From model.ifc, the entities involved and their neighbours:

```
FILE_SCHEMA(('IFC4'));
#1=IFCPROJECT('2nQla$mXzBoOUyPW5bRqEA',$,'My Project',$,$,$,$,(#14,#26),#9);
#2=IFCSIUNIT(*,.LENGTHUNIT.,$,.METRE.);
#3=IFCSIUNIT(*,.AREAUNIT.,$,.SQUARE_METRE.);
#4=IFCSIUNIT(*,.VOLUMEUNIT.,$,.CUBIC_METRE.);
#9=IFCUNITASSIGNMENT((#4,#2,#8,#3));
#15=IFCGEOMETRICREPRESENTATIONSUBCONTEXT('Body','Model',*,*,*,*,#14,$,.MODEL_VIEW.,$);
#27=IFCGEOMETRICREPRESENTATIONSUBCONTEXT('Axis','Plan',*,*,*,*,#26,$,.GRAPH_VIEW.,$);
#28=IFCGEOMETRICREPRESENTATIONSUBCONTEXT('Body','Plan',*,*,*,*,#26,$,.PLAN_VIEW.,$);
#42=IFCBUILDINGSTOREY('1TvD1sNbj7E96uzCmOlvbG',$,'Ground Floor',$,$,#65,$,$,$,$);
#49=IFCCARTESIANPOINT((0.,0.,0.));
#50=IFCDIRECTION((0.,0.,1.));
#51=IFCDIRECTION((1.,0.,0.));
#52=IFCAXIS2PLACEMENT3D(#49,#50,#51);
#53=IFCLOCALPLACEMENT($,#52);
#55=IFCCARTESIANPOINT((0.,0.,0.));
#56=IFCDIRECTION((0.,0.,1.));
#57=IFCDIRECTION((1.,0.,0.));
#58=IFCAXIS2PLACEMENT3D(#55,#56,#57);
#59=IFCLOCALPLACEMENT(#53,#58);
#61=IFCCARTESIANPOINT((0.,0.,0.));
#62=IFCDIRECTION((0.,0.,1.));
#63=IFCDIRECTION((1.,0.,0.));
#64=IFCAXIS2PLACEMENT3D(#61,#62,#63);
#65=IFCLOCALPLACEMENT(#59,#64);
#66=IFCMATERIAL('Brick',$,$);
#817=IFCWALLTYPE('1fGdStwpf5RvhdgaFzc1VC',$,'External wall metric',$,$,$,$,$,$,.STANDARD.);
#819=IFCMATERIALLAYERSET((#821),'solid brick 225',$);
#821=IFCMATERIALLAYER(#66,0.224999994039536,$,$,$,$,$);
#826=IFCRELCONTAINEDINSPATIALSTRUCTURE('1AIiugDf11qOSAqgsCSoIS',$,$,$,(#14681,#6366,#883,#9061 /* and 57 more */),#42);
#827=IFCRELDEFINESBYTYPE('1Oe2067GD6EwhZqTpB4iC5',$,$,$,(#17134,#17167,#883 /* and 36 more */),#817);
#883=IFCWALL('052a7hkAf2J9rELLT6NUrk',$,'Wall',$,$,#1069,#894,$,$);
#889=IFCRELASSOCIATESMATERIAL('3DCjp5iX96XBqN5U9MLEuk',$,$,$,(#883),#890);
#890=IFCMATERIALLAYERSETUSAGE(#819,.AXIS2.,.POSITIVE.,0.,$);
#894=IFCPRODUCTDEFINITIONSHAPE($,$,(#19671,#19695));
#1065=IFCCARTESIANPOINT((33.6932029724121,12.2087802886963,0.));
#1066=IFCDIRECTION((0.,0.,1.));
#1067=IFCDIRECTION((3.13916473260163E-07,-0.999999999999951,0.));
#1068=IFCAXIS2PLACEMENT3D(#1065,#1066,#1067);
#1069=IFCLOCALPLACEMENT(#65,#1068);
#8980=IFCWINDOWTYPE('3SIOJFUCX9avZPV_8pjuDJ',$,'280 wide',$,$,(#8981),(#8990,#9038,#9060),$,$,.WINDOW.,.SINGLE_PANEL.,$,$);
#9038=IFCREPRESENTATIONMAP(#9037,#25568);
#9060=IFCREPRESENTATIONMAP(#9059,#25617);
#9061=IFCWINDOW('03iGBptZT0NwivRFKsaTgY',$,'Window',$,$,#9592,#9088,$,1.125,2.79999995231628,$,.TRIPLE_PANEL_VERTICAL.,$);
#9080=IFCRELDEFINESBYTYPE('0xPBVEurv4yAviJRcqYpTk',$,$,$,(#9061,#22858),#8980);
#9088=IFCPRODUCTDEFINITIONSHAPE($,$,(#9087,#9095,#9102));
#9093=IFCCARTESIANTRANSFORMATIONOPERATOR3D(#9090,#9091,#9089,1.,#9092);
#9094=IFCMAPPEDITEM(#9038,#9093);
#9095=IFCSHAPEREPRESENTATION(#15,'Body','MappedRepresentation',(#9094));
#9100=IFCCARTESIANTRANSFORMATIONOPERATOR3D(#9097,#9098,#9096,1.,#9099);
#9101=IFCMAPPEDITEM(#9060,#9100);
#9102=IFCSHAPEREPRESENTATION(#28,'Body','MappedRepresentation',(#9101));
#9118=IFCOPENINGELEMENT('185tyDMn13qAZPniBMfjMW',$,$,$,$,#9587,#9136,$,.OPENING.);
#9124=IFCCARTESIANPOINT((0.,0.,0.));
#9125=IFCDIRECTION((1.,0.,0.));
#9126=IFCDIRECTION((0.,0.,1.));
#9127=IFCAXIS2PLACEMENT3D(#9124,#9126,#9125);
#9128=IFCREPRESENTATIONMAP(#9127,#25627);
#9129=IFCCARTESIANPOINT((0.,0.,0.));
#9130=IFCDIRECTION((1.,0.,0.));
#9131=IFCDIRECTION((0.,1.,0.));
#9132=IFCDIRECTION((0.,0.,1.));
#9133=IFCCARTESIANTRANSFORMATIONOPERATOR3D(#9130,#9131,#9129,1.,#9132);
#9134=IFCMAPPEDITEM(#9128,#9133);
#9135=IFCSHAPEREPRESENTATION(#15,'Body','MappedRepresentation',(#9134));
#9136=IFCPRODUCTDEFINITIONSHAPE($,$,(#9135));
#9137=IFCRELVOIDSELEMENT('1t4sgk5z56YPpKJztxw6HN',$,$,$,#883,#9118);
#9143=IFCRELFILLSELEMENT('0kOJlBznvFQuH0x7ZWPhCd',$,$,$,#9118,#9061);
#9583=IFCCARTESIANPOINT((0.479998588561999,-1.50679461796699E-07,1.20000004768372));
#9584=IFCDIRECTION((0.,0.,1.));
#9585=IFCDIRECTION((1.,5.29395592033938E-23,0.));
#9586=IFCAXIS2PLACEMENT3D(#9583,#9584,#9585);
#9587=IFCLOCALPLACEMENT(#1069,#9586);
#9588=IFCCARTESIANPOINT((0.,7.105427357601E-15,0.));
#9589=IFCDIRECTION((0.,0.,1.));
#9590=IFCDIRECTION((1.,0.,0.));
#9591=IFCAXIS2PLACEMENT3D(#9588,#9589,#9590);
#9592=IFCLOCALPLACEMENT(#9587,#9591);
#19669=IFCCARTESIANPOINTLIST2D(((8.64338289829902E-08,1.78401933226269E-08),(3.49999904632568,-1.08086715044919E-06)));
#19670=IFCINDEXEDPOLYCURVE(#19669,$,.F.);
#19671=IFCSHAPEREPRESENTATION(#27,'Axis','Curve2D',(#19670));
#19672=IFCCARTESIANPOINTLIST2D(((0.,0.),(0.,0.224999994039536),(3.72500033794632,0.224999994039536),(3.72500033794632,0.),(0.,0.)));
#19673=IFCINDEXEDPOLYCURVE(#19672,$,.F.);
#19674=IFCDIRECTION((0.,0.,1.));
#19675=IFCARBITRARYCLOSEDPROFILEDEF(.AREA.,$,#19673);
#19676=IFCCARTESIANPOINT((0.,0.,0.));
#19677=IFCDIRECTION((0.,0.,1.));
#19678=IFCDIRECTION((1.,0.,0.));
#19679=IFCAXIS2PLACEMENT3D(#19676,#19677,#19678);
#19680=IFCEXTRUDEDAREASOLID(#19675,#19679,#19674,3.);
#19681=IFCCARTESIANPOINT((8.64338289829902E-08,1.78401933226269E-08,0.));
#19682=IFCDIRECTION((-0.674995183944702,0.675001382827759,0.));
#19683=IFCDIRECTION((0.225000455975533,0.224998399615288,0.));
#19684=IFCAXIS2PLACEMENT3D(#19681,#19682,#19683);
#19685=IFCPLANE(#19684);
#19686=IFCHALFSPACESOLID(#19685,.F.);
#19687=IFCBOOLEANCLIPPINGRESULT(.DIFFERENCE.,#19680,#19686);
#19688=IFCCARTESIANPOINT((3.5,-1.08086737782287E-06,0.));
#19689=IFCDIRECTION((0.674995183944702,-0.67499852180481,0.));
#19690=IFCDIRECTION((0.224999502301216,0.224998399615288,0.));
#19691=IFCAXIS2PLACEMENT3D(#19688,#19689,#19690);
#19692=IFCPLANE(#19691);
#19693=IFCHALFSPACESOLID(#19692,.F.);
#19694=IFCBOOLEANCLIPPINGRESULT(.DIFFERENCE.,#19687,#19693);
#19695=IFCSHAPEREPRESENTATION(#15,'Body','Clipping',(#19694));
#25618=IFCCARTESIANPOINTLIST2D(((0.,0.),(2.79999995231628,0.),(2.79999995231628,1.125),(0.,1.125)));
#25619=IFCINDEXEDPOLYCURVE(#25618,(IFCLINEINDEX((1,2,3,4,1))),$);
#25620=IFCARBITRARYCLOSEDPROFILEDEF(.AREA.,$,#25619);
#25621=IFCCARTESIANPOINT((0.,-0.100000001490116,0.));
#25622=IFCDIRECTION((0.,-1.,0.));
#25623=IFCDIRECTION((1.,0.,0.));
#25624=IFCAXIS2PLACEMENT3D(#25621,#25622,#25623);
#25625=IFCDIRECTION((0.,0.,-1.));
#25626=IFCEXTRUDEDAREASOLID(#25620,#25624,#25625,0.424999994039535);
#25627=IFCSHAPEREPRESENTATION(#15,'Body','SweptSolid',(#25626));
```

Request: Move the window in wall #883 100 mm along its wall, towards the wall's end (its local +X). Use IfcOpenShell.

```python
import ifcopenshell
import ifcopenshell.api.geometry
import ifcopenshell.util.placement
import ifcopenshell.util.unit

model = ifcopenshell.open("model.ifc")
unit_scale = ifcopenshell.util.unit.calculate_unit_scale(model)

window = model.by_guid("03iGBptZT0NwivRFKsaTgY")
opening = window.FillsVoids[0].RelatingOpeningElement
wall = opening.VoidsElements[0].RelatingBuildingElement

wall_matrix = ifcopenshell.util.placement.get_local_placement(wall.ObjectPlacement)
shift = wall_matrix[:3, 0] * 0.1 / unit_scale
before = ifcopenshell.util.placement.get_local_placement(window.ObjectPlacement)[:3, 3].copy()

# The window is placed relative to its opening, so it follows when the opening moves.
matrix = ifcopenshell.util.placement.get_local_placement(opening.ObjectPlacement)
matrix[:3, 3] += shift
ifcopenshell.api.geometry.edit_object_placement(
    model, product=opening, matrix=matrix, is_si=False, should_transform_children=True
)

after = ifcopenshell.util.placement.get_local_placement(window.ObjectPlacement)[:3, 3]
print("window moved by", (after - before).round(3) + 0.0)

model.write("model_v2.ifc")
```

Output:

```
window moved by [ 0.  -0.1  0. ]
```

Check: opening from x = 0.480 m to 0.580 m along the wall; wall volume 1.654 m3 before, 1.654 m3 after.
